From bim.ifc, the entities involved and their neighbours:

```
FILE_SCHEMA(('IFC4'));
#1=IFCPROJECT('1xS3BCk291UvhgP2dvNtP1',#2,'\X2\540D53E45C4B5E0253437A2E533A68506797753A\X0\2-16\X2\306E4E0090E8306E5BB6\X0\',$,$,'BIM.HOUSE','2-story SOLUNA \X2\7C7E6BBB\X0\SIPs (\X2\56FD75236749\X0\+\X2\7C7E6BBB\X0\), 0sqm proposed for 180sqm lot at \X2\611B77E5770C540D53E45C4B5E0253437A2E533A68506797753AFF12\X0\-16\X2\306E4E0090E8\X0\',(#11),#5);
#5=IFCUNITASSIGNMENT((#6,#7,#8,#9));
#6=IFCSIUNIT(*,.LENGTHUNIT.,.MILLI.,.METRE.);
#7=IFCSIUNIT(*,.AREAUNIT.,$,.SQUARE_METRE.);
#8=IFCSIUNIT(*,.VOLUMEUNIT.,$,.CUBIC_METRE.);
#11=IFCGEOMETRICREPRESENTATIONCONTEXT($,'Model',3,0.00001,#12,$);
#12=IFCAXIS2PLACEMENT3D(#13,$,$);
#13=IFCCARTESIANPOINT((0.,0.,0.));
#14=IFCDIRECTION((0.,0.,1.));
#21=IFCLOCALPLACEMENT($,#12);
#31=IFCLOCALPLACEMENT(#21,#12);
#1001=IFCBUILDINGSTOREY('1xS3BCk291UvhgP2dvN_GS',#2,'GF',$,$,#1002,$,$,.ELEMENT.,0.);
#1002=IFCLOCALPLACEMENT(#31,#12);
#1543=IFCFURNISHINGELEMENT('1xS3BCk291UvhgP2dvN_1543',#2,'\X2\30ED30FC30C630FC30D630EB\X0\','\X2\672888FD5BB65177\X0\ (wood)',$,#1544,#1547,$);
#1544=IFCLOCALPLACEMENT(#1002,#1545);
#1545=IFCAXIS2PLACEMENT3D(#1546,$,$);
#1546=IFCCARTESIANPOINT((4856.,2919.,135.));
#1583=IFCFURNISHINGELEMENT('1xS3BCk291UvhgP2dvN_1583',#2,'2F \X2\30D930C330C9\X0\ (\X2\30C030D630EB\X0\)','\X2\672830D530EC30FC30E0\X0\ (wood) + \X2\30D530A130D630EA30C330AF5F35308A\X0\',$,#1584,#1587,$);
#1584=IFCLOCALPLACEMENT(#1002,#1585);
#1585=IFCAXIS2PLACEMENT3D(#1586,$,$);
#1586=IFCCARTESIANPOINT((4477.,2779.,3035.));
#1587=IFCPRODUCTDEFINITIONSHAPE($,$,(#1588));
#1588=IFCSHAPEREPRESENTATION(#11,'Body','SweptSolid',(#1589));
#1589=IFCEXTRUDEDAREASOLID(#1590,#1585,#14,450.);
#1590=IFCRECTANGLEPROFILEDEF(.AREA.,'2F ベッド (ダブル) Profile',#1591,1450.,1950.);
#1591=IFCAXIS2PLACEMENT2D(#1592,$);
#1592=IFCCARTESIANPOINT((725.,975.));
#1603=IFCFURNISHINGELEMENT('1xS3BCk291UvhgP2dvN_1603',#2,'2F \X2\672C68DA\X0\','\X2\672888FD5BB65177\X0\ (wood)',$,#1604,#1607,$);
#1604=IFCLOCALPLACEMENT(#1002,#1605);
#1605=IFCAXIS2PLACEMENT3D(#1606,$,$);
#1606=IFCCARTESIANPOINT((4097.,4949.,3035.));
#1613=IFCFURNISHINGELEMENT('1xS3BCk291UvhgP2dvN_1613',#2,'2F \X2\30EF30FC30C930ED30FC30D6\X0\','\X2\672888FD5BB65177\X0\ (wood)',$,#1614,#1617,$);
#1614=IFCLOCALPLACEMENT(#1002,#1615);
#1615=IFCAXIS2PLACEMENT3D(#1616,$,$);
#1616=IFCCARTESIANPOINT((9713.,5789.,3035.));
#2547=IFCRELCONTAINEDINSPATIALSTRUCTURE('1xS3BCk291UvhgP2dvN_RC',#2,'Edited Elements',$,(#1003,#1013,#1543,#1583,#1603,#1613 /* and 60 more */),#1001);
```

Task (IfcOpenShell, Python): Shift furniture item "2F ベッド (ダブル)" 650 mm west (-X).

```python
import ifcopenshell
import ifcopenshell.api.geometry
import ifcopenshell.util.placement
import ifcopenshell.util.unit

model = ifcopenshell.open("bim.ifc")
unit_scale = ifcopenshell.util.unit.calculate_unit_scale(model)

item = model.by_guid("1xS3BCk291UvhgP2dvN_1583")
matrix = ifcopenshell.util.placement.get_local_placement(item.ObjectPlacement)
matrix[0, 3] -= 0.65 / unit_scale
ifcopenshell.api.geometry.edit_object_placement(model, product=item, matrix=matrix, is_si=False)

print(ifcopenshell.util.placement.get_local_placement(item.ObjectPlacement).round(3) + 0.0)

model.write("bim_v2.ifc")
```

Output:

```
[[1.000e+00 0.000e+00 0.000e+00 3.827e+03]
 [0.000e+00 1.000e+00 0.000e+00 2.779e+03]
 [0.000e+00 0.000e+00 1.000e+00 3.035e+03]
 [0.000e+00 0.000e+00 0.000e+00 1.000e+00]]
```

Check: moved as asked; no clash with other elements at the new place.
